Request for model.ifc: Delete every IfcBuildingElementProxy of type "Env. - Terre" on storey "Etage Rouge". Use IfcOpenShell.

First a look at what the model holds.

```python
import ifcopenshell
import ifcopenshell.util.element

model = ifcopenshell.open("model.ifc")
print(model.schema)
storey = next(s for s in model.by_type("IfcBuildingStorey") if s.Name == "Etage Rouge")
proxies = [e for e in ifcopenshell.util.element.get_decomposition(storey) if e.is_a("IfcBuildingElementProxy")]
seen = {}
for e in proxies:
    element_type = ifcopenshell.util.element.get_type(e)
    name = element_type.Name if element_type not in (None, e) else None
    seen[name] = seen.get(name, 0) + 1
for name, count in sorted(seen.items(), key=str):
    print(count, "x", name)
```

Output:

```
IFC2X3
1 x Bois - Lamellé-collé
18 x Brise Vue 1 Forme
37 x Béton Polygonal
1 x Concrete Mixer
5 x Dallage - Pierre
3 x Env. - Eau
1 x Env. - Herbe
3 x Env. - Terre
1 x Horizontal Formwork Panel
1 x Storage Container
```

```python
import ifcopenshell
import ifcopenshell.api.root
import ifcopenshell.util.element

model = ifcopenshell.open("model.ifc")

storey = next(s for s in model.by_type("IfcBuildingStorey") if s.Name == "Etage Rouge")
proxies = [e for e in ifcopenshell.util.element.get_decomposition(storey) if e.is_a("IfcBuildingElementProxy")]
targets = [e for e in proxies if (t := ifcopenshell.util.element.get_type(e)) not in (None, e) and t.Name == "Env. - Terre"]

for e in targets:
    ifcopenshell.api.root.remove_product(model, product=e)
print(len(targets), "removed")

model.write("model-out.ifc")
```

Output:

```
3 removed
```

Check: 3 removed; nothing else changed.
